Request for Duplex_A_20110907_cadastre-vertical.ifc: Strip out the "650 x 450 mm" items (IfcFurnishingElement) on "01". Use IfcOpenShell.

First a look at what the model holds.

```python
import ifcopenshell
import ifcopenshell.util.element

model = ifcopenshell.open("Duplex_A_20110907_cadastre-vertical.ifc")
print(model.schema)
storey = next(s for s in model.by_type("IfcBuildingStorey") if s.Name == "01")
furniture = [e for e in ifcopenshell.util.element.get_decomposition(storey) if e.is_a("IfcFurnishingElement")]
seen = {}
for e in furniture:
    element_type = ifcopenshell.util.element.get_type(e)
    name = element_type.Name if element_type not in (None, e) else None
    seen[name] = seen.get(name, 0) + 1
for name, count in sorted(seen.items(), key=str):
    print(count, "x", name)
```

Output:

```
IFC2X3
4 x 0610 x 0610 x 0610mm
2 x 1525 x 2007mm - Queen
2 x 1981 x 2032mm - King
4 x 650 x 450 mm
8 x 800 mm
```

```python
import ifcopenshell
import ifcopenshell.api.root
import ifcopenshell.util.element

model = ifcopenshell.open("Duplex_A_20110907_cadastre-vertical.ifc")

storey = next(s for s in model.by_type("IfcBuildingStorey") if s.Name == "01")
furniture = [e for e in ifcopenshell.util.element.get_decomposition(storey) if e.is_a("IfcFurnishingElement")]
targets = [e for e in furniture if (t := ifcopenshell.util.element.get_type(e)) not in (None, e) and t.Name == "650 x 450 mm"]

for e in targets:
    ifcopenshell.api.root.remove_product(model, product=e)
print(len(targets), "removed")

model.write("Duplex_A_20110907_cadastre-vertical_rev.ifc")
```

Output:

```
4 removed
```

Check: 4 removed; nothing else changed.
